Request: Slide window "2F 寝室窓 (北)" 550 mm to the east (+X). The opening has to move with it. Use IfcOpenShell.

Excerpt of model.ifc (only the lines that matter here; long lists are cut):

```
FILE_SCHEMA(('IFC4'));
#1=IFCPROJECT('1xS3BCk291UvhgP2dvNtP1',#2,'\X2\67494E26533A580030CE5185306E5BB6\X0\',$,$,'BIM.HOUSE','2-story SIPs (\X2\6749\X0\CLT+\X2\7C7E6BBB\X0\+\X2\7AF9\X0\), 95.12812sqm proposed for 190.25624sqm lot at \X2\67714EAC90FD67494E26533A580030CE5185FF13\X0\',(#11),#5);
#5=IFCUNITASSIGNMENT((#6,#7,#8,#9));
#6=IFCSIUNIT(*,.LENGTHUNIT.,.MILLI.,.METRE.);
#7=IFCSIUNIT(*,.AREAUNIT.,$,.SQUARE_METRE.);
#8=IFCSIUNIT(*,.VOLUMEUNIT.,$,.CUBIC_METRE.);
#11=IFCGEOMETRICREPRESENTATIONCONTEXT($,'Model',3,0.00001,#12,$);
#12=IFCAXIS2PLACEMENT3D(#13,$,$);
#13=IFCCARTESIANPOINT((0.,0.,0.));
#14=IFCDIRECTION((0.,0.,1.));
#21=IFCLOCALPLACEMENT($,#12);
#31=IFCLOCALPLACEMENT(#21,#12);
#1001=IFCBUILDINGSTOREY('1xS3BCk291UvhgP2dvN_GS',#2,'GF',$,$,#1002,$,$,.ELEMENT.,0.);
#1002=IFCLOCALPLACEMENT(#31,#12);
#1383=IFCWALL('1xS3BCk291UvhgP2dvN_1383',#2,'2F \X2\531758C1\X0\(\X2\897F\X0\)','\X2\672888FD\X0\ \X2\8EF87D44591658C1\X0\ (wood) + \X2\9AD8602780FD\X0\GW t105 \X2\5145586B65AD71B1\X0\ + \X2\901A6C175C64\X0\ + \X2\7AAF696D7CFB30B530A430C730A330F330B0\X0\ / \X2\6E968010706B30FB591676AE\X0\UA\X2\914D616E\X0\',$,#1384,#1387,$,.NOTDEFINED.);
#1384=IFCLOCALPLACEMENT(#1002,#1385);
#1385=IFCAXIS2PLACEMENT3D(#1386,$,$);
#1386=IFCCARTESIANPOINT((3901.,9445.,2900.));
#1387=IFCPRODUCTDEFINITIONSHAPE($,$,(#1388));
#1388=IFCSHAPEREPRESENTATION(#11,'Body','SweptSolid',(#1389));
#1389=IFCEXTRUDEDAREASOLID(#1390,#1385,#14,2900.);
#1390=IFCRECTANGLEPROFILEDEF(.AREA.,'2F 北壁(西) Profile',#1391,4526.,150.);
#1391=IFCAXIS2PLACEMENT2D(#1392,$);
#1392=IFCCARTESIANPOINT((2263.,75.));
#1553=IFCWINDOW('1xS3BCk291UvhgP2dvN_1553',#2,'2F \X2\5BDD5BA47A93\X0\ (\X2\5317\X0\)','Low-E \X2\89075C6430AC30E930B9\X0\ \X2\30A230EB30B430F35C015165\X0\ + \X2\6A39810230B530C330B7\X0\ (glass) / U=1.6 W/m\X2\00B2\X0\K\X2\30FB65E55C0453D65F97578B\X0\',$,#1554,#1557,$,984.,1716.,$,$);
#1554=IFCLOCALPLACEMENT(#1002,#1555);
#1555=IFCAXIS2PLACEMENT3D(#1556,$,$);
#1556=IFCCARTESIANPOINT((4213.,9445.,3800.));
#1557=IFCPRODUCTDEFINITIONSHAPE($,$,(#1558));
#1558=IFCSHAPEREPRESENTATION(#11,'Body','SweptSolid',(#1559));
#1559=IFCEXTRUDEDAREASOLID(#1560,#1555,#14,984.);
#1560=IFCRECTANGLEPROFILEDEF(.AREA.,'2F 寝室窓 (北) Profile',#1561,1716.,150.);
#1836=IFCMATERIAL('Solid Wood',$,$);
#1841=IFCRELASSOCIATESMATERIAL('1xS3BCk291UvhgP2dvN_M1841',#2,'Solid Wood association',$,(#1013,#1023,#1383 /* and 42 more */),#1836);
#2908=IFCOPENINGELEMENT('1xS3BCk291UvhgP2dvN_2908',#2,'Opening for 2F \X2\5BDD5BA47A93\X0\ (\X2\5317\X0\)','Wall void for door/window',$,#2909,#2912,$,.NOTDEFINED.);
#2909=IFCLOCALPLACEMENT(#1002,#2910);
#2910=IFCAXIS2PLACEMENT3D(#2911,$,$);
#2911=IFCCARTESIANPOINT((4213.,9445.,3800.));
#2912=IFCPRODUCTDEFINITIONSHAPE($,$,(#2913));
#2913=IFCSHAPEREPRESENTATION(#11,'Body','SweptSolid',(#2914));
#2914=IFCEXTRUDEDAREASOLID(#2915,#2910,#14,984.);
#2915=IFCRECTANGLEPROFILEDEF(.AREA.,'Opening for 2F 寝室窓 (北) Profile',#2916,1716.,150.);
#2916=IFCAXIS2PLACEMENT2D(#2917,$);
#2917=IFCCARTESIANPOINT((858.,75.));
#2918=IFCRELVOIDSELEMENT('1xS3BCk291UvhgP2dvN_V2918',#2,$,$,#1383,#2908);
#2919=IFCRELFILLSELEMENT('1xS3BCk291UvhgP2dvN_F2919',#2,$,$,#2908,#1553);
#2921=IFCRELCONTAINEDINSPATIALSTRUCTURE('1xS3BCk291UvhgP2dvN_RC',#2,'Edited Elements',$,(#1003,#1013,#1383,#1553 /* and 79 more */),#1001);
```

```python
import ifcopenshell
import ifcopenshell.api.geometry
import ifcopenshell.util.placement
import ifcopenshell.util.unit

model = ifcopenshell.open("model.ifc")
unit_scale = ifcopenshell.util.unit.calculate_unit_scale(model)

window = model.by_guid("1xS3BCk291UvhgP2dvN_1553")
opening = window.FillsVoids[0].RelatingOpeningElement
wall = opening.VoidsElements[0].RelatingBuildingElement

wall_matrix = ifcopenshell.util.placement.get_local_placement(wall.ObjectPlacement)
shift = wall_matrix[:3, 0] * 0.55 / unit_scale
before = ifcopenshell.util.placement.get_local_placement(window.ObjectPlacement)[:3, 3].copy()

# The window is not placed relative to its opening, so move both.
for product in (opening, window):
    matrix = ifcopenshell.util.placement.get_local_placement(product.ObjectPlacement)
    matrix[:3, 3] += shift
    ifcopenshell.api.geometry.edit_object_placement(model, product=product, matrix=matrix, is_si=False)

after = ifcopenshell.util.placement.get_local_placement(window.ObjectPlacement)[:3, 3]
print("window moved by", (after - before).round(3) + 0.0)

model.write("model_v2.ifc")
```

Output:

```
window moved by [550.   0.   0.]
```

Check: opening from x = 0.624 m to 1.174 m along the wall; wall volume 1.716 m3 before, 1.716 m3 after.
